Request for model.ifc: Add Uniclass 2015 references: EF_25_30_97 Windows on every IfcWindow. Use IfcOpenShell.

First a look at what the model holds.

```python
import ifcopenshell

model = ifcopenshell.open("model.ifc")
print(model.schema)
print("classifications:", [c.Name for c in model.by_type("IfcClassification")])
for ifc_class in ("IfcDoor", "IfcRoof", "IfcStair", "IfcWall", "IfcWindow"):
    print(ifc_class, len(model.by_type(ifc_class)))
```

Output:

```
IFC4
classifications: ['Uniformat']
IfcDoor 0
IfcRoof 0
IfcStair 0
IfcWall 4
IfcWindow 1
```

```python
import ifcopenshell
import ifcopenshell.api.classification

model = ifcopenshell.open("model.ifc")

system = ifcopenshell.api.classification.add_classification(model, classification="Uniclass 2015")

codes = {
    "IfcWindow": ("EF_25_30_97", "Windows"),
}
for ifc_class, (code, name) in codes.items():
    products = model.by_type(ifc_class)
    ifcopenshell.api.classification.add_reference(
        model, products=products, classification=system, identification=code, name=name
    )
    print(code, len(products))

model.write("model_edited.ifc")
```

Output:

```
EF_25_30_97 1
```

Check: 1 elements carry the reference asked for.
